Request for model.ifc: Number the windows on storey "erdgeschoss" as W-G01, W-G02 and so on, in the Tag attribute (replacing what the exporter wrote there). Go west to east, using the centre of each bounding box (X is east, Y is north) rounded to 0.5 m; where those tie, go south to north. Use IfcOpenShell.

First a look at what the model holds.

```python
import ifcopenshell
import ifcopenshell.util.element
import ifcopenshell.util.placement

model = ifcopenshell.open("model.ifc")
print(model.schema)
storey = next(s for s in model.by_type("IfcBuildingStorey") if s.Name == "erdgeschoss")
windows = [e for e in ifcopenshell.util.element.get_decomposition(storey) if e.is_a("IfcWindow")]
for e in sorted(windows, key=lambda e: e.id()):
    origin = ifcopenshell.util.placement.get_local_placement(e.ObjectPlacement)[:3, 3]
    print(e.id(), e.Tag, e.Name, origin.round(2) + 0.0, sep=" | ")
```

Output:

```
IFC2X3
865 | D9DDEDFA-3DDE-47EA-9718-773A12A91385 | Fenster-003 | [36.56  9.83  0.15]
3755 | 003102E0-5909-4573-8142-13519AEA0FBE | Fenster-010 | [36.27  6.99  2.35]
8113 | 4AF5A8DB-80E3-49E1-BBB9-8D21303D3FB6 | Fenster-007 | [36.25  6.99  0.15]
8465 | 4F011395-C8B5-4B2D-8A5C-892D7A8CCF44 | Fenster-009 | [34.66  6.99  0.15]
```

```python
import ifcopenshell
import ifcopenshell.geom
import ifcopenshell.util.element
import ifcopenshell.util.shape

model = ifcopenshell.open("model.ifc")
settings = ifcopenshell.geom.settings()
settings.set("use-world-coords", True)


def centre(element):
    shape = ifcopenshell.geom.create_shape(settings, element)
    return ifcopenshell.util.shape.get_bbox_centroid(shape.geometry)


storey = next(s for s in model.by_type("IfcBuildingStorey") if s.Name == "erdgeschoss")
windows = [e for e in ifcopenshell.util.element.get_decomposition(storey) if e.is_a("IfcWindow")]

# Insertion points can sit at a corner or the storey origin, so sort by the geometry (in metres).
centres = {e: centre(e) for e in windows}
windows.sort(key=lambda e: (round(centres[e][0] / 0.5), centres[e][1]))

for i, e in enumerate(windows, start=1):
    number = f"W-G{i:02d}"
    e.Tag = number
    print(e.id(), number)

model.write("model_rev.ifc")
```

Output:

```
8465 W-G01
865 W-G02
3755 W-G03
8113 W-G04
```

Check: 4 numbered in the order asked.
